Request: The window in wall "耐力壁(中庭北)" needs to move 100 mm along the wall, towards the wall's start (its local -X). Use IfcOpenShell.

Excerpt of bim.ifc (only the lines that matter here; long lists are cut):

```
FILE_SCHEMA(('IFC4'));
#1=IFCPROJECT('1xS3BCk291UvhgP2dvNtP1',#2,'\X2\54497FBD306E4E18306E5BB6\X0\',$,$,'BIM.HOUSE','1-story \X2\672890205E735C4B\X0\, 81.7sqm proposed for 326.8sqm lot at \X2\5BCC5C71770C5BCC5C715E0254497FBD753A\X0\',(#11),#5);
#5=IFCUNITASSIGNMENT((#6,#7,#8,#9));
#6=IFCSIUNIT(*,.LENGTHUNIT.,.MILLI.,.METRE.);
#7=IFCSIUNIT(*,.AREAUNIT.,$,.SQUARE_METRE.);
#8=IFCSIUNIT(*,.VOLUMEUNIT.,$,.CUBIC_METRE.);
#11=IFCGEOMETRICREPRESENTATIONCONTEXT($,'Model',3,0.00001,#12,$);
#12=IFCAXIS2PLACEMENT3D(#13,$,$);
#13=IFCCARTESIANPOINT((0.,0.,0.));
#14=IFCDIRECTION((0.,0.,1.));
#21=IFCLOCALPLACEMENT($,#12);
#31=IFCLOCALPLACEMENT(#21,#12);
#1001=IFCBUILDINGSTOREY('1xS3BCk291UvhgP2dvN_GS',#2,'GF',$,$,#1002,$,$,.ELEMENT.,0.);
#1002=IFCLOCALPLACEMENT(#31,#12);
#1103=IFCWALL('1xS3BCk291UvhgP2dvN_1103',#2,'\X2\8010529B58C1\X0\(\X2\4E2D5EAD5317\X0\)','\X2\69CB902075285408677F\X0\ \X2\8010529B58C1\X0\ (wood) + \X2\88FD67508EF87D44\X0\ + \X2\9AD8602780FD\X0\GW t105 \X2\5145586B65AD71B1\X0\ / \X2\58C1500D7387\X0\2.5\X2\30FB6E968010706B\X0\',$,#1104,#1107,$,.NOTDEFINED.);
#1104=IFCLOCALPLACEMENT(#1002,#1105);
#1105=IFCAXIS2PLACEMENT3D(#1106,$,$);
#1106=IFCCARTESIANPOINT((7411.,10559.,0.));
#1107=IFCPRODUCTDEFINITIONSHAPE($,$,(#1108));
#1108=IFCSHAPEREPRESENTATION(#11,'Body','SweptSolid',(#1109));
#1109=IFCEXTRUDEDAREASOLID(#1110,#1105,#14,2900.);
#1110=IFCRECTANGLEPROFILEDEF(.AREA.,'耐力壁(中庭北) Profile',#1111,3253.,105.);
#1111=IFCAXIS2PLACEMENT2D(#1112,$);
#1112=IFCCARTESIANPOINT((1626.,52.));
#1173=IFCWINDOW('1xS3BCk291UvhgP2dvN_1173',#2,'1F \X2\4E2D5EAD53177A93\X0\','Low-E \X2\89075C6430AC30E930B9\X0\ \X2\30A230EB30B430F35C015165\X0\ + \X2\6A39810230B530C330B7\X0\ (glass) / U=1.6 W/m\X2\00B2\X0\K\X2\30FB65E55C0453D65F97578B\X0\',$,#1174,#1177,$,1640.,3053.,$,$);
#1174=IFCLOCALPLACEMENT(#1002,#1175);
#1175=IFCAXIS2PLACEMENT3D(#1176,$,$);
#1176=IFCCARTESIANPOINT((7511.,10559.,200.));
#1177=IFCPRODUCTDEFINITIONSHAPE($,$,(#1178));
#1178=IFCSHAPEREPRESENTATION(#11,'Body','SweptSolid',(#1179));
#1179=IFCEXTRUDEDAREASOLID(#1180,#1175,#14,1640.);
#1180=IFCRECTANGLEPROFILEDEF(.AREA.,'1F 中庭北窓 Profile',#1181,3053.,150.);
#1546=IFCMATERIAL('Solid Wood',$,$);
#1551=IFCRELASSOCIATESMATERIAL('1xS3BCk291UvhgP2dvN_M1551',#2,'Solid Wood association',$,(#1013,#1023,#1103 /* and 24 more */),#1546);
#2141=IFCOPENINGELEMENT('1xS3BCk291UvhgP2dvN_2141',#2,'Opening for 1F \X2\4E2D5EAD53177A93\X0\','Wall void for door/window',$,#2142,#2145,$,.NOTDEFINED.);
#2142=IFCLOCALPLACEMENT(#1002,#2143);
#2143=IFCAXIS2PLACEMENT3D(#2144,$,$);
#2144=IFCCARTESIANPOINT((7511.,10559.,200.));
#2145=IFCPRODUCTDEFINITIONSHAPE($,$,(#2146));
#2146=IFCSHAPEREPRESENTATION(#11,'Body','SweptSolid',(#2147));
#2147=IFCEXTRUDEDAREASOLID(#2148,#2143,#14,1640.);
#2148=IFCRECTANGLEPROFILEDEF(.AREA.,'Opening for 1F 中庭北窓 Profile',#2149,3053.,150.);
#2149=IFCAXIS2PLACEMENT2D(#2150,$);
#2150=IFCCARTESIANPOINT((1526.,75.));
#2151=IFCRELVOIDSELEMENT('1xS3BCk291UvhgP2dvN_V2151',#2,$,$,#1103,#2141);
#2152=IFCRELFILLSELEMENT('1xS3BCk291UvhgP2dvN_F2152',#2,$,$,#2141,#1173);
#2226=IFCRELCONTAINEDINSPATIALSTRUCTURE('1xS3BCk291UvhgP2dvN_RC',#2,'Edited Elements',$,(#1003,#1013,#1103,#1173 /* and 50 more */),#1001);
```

```python
import ifcopenshell
import ifcopenshell.api.geometry
import ifcopenshell.util.placement

model = ifcopenshell.open("bim.ifc")

window = model.by_guid("1xS3BCk291UvhgP2dvN_1173")
opening = window.FillsVoids[0].RelatingOpeningElement
wall = opening.VoidsElements[0].RelatingBuildingElement

wall_matrix = ifcopenshell.util.placement.get_local_placement(wall.ObjectPlacement)
shift = wall_matrix[:3, 0] * -100.0
before = ifcopenshell.util.placement.get_local_placement(window.ObjectPlacement)[:3, 3].copy()

# The window is not placed relative to its opening, so move both.
for product in (opening, window):
    matrix = ifcopenshell.util.placement.get_local_placement(product.ObjectPlacement)
    matrix[:3, 3] += shift
    ifcopenshell.api.geometry.edit_object_placement(model, product=product, matrix=matrix, is_si=False)

after = ifcopenshell.util.placement.get_local_placement(window.ObjectPlacement)[:3, 3]
print("window moved by", (after - before).round(3) + 0.0)

model.write("bim_updated.ifc")
```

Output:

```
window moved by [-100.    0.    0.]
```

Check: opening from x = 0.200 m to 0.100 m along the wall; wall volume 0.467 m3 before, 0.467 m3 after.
